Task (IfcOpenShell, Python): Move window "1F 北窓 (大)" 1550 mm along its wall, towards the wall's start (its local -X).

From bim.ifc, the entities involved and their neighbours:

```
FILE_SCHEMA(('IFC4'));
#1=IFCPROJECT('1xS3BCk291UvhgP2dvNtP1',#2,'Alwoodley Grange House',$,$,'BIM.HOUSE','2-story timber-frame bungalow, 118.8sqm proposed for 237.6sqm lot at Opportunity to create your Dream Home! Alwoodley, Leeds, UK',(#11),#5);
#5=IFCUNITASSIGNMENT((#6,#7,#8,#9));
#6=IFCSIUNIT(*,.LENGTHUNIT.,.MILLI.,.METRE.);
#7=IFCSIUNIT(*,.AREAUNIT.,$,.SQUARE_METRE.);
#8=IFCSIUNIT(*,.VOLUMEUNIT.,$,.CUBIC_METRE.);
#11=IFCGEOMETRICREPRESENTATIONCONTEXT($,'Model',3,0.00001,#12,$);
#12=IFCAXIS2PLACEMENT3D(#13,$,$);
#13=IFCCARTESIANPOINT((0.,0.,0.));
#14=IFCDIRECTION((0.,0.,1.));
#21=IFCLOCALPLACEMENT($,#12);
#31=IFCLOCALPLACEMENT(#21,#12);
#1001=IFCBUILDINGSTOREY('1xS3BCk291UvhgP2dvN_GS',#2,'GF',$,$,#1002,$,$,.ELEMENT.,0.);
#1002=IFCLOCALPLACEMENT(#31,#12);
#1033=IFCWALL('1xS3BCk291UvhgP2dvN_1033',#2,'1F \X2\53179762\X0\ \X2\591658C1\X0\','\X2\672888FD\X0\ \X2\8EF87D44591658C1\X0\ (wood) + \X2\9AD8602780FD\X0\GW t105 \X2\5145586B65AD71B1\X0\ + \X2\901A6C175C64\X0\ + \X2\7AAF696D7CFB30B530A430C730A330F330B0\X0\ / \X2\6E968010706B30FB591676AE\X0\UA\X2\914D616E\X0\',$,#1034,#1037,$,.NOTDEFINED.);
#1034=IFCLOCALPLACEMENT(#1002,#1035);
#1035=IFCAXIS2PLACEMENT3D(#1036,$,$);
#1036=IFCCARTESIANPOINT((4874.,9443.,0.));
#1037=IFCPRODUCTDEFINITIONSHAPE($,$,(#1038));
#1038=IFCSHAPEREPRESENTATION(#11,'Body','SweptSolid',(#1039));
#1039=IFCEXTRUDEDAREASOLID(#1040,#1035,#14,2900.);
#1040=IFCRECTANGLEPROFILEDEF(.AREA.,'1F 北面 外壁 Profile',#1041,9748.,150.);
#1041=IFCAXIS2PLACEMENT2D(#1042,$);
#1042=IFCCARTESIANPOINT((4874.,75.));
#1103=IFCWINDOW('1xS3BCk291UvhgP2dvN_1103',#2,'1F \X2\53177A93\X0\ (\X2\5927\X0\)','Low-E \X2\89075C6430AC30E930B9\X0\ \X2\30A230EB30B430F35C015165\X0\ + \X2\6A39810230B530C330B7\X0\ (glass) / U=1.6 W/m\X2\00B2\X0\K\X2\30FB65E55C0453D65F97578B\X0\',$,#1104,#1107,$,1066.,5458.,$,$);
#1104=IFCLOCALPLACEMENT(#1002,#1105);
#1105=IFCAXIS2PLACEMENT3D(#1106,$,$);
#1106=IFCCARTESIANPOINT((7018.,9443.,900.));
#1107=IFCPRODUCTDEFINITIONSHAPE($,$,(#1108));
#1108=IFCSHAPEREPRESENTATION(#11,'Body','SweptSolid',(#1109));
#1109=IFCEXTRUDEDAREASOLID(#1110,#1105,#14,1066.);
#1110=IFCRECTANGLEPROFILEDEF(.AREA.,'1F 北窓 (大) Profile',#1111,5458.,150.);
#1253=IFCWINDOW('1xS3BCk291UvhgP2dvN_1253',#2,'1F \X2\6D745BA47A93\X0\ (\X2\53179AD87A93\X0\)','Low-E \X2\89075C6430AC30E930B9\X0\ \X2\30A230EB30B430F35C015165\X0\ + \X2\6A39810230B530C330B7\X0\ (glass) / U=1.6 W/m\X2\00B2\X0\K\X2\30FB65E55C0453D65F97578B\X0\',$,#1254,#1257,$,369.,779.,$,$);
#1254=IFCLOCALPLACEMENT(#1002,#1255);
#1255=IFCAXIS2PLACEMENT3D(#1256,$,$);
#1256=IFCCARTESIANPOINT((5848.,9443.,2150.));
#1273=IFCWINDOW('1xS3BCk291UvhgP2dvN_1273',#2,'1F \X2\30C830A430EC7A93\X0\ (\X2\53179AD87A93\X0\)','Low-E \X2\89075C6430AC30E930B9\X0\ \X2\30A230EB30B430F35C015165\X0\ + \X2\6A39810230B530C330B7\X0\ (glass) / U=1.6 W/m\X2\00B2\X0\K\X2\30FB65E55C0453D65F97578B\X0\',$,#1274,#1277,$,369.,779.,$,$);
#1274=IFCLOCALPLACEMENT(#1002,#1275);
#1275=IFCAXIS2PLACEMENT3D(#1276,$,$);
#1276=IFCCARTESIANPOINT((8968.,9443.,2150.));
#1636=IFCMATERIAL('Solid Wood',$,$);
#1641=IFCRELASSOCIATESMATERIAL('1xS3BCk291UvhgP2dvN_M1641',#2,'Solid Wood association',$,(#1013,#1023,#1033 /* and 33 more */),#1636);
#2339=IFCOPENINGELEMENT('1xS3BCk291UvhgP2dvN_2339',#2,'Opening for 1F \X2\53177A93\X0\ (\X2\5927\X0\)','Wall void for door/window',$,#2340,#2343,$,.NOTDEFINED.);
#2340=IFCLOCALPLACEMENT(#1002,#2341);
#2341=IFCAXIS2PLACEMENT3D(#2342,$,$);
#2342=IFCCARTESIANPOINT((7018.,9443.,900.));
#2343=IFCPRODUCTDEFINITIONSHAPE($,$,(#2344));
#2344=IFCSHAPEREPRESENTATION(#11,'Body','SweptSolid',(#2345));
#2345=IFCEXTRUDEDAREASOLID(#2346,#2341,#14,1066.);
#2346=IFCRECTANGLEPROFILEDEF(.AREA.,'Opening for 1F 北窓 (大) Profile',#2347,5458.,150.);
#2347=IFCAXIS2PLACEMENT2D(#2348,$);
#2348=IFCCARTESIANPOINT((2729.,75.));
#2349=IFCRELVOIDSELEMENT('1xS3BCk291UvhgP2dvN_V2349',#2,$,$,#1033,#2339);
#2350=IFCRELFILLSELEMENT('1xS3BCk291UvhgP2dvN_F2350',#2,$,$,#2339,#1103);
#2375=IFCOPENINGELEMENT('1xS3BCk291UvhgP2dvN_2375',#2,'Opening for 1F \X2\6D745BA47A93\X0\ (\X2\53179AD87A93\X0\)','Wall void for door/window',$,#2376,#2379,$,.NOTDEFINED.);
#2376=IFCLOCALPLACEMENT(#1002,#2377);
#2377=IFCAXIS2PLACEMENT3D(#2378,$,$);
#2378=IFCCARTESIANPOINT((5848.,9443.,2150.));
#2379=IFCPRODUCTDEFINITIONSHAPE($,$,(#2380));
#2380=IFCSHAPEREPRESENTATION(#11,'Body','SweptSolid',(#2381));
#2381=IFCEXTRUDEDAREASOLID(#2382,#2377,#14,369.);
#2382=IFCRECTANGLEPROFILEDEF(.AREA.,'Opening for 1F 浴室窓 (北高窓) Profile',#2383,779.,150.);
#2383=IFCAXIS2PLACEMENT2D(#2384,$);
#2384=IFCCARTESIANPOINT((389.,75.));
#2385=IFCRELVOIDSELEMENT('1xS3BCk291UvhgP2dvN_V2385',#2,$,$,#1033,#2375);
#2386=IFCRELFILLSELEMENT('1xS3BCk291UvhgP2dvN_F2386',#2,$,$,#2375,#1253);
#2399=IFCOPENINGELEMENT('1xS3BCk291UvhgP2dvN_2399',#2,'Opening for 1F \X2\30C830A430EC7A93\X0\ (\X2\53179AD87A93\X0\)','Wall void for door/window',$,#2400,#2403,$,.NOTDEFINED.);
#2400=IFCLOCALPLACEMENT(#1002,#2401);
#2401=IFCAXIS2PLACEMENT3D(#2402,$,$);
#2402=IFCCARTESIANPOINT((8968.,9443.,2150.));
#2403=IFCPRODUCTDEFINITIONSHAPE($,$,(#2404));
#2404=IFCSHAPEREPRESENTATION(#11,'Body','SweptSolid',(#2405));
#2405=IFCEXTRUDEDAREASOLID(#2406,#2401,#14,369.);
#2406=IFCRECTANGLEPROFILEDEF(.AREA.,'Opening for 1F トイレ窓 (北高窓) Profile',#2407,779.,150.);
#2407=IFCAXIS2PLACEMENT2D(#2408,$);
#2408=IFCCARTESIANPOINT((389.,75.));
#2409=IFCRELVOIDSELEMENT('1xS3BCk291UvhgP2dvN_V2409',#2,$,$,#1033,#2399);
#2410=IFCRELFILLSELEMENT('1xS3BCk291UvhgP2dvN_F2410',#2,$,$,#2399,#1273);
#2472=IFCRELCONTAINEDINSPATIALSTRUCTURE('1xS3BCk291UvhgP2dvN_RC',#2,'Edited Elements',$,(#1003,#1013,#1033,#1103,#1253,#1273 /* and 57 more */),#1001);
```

```python
import ifcopenshell
import ifcopenshell.api.geometry
import ifcopenshell.util.placement

model = ifcopenshell.open("bim.ifc")

window = model.by_guid("1xS3BCk291UvhgP2dvN_1103")
opening = window.FillsVoids[0].RelatingOpeningElement
wall = opening.VoidsElements[0].RelatingBuildingElement

wall_matrix = ifcopenshell.util.placement.get_local_placement(wall.ObjectPlacement)
shift = wall_matrix[:3, 0] * -1550.0
before = ifcopenshell.util.placement.get_local_placement(window.ObjectPlacement)[:3, 3].copy()

# The window is not placed relative to its opening, so move both.
for product in (opening, window):
    matrix = ifcopenshell.util.placement.get_local_placement(product.ObjectPlacement)
    matrix[:3, 3] += shift
    ifcopenshell.api.geometry.edit_object_placement(model, product=product, matrix=matrix, is_si=False)

after = ifcopenshell.util.placement.get_local_placement(window.ObjectPlacement)[:3, 3]
print("window moved by", (after - before).round(3) + 0.0)

model.write("bim_updated.ifc")
```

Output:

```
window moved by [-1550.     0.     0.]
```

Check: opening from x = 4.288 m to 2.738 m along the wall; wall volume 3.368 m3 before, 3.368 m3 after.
